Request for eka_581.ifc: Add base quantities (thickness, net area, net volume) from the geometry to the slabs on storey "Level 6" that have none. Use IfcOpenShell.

First a look at what the model holds.

```python
import ifcopenshell
import ifcopenshell.util.element
import ifcopenshell.util.unit

model = ifcopenshell.open("eka_581.ifc")
print(model.schema)
for unit_type in ("LENGTHUNIT", "AREAUNIT", "VOLUMEUNIT"):
    print(unit_type, ifcopenshell.util.unit.calculate_unit_scale(model, unit_type))
storey = next(s for s in model.by_type("IfcBuildingStorey") if s.Name == "Level 6")
slabs = [e for e in ifcopenshell.util.element.get_decomposition(storey) if e.is_a("IfcSlab")]
for e in sorted(slabs, key=lambda e: e.id()):
    print(e.id(), e.is_a(), e.Name, list(ifcopenshell.util.element.get_psets(e, qtos_only=True)), sep=" | ")
```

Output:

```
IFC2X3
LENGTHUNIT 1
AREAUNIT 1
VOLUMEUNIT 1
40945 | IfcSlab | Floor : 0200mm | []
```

```python
import ifcopenshell
import ifcopenshell.api.pset
import ifcopenshell.geom
import ifcopenshell.util.element
import ifcopenshell.util.shape
import ifcopenshell.util.unit

model = ifcopenshell.open("eka_581.ifc")
unit_scale = ifcopenshell.util.unit.calculate_unit_scale(model)
area_scale = ifcopenshell.util.unit.calculate_unit_scale(model, "AREAUNIT")
volume_scale = ifcopenshell.util.unit.calculate_unit_scale(model, "VOLUMEUNIT")
settings = ifcopenshell.geom.settings()

storey = next(s for s in model.by_type("IfcBuildingStorey") if s.Name == "Level 6")
slabs = [e for e in ifcopenshell.util.element.get_decomposition(storey) if e.is_a("IfcSlab")]

for e in sorted(slabs, key=lambda e: e.id()):
    if ifcopenshell.util.element.get_psets(e, qtos_only=True, should_inherit=False):
        continue
    # Geometry comes back in metres, in the element's own axes.
    shape = ifcopenshell.geom.create_shape(settings, e)
    values = {
        "Width": ifcopenshell.util.shape.get_z(shape.geometry) / unit_scale,
        "NetArea": ifcopenshell.util.shape.get_footprint_area(shape.geometry) / area_scale,
        "NetVolume": ifcopenshell.util.shape.get_volume(shape.geometry) / volume_scale,
    }
    qto = ifcopenshell.api.pset.add_qto(model, product=e, name="BaseQuantities")
    ifcopenshell.api.pset.edit_qto(model, qto=qto, properties=values)
    print(e.id(), {k: round(v, 3) for k, v in values.items()})

model.write("eka_581-out.ifc")
```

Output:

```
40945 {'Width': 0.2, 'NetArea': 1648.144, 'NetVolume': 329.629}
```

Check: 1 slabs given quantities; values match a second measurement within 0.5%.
